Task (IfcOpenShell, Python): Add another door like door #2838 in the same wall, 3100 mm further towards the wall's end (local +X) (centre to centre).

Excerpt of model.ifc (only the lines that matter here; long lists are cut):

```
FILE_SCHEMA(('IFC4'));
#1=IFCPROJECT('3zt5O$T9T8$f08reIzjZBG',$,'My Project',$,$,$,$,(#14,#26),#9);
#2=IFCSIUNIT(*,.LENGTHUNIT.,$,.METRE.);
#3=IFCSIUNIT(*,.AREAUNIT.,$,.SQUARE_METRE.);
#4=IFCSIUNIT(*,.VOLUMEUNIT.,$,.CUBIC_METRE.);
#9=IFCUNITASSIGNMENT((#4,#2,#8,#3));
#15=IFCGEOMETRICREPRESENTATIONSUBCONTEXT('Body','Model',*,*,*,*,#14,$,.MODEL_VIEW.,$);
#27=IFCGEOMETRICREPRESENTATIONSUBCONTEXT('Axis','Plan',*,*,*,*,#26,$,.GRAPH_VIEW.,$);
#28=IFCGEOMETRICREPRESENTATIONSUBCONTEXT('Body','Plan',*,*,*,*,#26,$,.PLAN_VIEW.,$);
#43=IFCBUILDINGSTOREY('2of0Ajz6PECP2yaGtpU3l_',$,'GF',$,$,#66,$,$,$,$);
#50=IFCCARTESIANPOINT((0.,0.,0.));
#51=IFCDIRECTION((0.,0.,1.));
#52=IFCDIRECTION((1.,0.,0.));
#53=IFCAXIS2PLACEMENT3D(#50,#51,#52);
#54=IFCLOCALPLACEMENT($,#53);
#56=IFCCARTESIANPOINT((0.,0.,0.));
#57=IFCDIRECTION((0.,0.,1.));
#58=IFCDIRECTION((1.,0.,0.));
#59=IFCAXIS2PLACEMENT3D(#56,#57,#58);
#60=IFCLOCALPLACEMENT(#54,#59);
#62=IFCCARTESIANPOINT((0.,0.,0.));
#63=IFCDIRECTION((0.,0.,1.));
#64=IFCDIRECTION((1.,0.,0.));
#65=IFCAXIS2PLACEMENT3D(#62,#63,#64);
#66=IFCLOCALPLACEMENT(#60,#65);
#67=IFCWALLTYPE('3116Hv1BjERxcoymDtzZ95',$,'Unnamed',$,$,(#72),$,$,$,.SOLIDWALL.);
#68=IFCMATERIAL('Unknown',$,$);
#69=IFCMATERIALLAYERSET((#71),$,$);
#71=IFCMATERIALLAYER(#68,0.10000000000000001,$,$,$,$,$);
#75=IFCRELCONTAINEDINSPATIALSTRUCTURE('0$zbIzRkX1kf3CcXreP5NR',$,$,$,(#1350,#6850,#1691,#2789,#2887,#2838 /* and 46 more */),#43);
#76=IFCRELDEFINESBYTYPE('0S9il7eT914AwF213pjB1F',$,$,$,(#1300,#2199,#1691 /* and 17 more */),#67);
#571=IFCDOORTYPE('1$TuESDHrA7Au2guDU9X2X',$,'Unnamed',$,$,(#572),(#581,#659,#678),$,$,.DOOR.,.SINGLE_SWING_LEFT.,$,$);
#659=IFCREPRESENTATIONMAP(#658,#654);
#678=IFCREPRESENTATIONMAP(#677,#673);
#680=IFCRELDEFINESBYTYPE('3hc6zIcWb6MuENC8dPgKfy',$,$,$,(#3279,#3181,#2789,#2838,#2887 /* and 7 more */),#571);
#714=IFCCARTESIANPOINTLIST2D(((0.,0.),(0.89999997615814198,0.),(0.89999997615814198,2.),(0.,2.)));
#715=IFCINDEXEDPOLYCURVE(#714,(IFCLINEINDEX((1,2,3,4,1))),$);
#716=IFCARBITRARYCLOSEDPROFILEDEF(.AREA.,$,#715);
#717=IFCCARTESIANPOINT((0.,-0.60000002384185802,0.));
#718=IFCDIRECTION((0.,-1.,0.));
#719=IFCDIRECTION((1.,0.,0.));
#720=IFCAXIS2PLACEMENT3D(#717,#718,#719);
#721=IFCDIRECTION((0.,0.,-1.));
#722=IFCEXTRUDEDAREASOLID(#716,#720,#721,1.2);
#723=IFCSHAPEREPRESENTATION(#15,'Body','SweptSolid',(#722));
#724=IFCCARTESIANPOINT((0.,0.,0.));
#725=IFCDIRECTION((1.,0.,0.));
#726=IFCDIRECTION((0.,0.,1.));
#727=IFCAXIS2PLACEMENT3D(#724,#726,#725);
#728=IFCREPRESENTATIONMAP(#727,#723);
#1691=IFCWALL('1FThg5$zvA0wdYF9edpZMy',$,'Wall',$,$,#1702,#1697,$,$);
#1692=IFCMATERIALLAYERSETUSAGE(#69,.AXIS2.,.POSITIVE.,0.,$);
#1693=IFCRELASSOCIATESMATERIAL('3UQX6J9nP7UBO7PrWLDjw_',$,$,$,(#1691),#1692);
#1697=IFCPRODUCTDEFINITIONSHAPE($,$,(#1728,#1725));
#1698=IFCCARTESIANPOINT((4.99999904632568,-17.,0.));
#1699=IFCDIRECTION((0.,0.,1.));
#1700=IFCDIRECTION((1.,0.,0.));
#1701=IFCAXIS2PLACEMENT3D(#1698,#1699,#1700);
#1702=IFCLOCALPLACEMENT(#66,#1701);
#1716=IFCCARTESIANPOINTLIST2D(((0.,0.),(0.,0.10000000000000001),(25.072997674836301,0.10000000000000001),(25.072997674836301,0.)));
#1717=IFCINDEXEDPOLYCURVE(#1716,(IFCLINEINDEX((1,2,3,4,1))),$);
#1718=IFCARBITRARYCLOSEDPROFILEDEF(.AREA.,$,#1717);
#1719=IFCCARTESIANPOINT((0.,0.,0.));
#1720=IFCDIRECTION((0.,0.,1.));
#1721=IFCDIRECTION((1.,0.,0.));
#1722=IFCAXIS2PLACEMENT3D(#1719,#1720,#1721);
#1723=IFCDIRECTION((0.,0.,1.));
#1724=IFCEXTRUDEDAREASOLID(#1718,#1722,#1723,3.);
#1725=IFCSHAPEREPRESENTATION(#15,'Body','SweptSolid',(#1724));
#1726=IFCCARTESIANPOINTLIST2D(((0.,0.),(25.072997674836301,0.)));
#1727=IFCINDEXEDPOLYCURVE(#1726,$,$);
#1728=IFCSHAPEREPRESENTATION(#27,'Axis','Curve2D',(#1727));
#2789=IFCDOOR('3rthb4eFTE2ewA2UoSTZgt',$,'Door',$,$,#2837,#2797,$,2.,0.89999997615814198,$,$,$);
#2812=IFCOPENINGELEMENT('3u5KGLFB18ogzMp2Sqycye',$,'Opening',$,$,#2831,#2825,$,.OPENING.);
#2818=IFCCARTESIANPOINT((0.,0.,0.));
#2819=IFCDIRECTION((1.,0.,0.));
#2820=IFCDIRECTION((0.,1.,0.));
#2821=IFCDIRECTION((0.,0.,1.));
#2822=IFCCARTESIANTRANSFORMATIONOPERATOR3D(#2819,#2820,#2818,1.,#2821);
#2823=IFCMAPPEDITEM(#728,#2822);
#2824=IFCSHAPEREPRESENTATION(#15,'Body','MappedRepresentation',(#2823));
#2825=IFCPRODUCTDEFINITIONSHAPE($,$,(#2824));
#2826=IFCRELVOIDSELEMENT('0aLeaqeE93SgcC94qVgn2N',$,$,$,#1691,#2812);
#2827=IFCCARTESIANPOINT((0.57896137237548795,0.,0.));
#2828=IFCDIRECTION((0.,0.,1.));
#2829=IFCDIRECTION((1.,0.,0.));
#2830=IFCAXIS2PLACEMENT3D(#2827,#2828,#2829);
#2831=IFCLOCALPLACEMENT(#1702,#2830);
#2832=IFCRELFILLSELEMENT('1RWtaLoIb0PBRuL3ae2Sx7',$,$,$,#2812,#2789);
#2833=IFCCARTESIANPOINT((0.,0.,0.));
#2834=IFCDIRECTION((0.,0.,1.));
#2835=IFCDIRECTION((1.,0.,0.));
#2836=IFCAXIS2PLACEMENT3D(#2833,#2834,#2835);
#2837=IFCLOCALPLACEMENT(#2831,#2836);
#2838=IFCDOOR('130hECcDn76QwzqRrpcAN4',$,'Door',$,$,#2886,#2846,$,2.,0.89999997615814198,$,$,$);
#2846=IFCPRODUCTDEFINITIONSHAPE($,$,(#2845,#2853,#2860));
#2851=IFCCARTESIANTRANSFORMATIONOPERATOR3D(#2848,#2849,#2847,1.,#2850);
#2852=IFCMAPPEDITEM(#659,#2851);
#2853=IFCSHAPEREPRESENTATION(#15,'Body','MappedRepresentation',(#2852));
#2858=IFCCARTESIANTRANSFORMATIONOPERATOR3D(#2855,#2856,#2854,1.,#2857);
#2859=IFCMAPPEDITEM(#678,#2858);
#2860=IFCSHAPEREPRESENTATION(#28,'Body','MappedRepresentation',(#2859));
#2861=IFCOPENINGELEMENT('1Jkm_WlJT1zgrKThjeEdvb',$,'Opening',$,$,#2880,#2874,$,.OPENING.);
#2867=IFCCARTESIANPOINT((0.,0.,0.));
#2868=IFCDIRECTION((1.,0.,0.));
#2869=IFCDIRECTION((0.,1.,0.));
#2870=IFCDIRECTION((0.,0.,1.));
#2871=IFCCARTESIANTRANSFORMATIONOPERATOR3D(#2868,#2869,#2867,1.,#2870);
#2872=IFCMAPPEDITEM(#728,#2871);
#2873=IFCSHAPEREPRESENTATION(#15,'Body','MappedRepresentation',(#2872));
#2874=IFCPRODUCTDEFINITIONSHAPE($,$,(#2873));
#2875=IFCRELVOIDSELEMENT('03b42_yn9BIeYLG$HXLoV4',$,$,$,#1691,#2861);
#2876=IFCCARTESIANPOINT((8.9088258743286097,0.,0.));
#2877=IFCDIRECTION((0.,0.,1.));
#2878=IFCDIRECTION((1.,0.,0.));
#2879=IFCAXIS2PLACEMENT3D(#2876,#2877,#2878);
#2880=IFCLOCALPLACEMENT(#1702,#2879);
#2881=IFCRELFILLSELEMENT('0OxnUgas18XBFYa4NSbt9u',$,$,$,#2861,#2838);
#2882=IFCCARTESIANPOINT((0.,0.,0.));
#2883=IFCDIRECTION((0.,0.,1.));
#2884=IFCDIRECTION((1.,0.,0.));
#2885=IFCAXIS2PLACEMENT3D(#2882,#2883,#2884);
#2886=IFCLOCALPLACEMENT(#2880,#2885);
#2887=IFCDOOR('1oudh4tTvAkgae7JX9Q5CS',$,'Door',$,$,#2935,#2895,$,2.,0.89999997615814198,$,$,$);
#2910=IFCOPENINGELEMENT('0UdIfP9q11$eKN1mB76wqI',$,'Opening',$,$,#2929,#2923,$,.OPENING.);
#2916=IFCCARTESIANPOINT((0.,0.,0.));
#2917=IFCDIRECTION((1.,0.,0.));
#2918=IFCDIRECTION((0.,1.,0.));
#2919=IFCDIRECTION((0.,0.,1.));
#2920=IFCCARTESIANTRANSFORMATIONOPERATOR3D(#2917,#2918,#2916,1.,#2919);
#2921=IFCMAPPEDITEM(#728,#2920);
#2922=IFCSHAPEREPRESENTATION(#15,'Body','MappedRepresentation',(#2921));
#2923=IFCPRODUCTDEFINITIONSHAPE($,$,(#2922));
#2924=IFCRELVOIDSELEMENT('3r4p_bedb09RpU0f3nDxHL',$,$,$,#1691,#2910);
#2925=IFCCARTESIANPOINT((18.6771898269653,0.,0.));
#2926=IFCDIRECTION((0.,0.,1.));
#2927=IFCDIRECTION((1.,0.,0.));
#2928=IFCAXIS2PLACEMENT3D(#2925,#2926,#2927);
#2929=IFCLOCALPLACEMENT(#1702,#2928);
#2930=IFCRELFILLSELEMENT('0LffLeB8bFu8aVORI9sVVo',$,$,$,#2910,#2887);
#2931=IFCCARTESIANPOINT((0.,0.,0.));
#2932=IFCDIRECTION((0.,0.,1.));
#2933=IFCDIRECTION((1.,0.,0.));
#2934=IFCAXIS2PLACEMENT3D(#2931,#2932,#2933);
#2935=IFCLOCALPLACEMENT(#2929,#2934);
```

```python
import ifcopenshell
import ifcopenshell.api.feature
import ifcopenshell.api.geometry
import ifcopenshell.api.root
import ifcopenshell.geom
import ifcopenshell.util.element
import ifcopenshell.util.placement
import ifcopenshell.util.shape

model = ifcopenshell.open("model.ifc")
settings = ifcopenshell.geom.settings()


def volume(element):
    """Net volume in cubic metres, openings subtracted."""
    shape = ifcopenshell.geom.create_shape(settings, element)
    return ifcopenshell.util.shape.get_volume(shape.geometry)


door = model.by_guid("130hECcDn76QwzqRrpcAN4")
opening = door.FillsVoids[0].RelatingOpeningElement
wall = opening.VoidsElements[0].RelatingBuildingElement
before = volume(wall)
shift = ifcopenshell.util.placement.get_local_placement(wall.ObjectPlacement)[:3, 0] * 3.1

# copy_class copies the void relationship, type, container and properties, but no geometry.
new_opening = ifcopenshell.api.root.copy_class(model, product=opening)
new_opening.Representation = ifcopenshell.util.element.copy_deep(
    model, opening.Representation, exclude=["IfcGeometricRepresentationContext", "IfcRepresentationMap"]
)
new_door = ifcopenshell.api.root.copy_class(model, product=door)
new_door.Representation = ifcopenshell.util.element.copy_deep(
    model, door.Representation, exclude=["IfcGeometricRepresentationContext", "IfcRepresentationMap"]
)
ifcopenshell.api.feature.add_filling(model, opening=new_opening, element=new_door)

for old, new in ((opening, new_opening), (door, new_door)):
    matrix = ifcopenshell.util.placement.get_local_placement(old.ObjectPlacement)
    matrix[:3, 3] += shift
    ifcopenshell.api.geometry.edit_object_placement(model, product=new, matrix=matrix, is_si=False)

after = volume(wall)

print(f"wall volume {before:.3f} -> {after:.3f} m3")

model.write("model-out.ifc")
```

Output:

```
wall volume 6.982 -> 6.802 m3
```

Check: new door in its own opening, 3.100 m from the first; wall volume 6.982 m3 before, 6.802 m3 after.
